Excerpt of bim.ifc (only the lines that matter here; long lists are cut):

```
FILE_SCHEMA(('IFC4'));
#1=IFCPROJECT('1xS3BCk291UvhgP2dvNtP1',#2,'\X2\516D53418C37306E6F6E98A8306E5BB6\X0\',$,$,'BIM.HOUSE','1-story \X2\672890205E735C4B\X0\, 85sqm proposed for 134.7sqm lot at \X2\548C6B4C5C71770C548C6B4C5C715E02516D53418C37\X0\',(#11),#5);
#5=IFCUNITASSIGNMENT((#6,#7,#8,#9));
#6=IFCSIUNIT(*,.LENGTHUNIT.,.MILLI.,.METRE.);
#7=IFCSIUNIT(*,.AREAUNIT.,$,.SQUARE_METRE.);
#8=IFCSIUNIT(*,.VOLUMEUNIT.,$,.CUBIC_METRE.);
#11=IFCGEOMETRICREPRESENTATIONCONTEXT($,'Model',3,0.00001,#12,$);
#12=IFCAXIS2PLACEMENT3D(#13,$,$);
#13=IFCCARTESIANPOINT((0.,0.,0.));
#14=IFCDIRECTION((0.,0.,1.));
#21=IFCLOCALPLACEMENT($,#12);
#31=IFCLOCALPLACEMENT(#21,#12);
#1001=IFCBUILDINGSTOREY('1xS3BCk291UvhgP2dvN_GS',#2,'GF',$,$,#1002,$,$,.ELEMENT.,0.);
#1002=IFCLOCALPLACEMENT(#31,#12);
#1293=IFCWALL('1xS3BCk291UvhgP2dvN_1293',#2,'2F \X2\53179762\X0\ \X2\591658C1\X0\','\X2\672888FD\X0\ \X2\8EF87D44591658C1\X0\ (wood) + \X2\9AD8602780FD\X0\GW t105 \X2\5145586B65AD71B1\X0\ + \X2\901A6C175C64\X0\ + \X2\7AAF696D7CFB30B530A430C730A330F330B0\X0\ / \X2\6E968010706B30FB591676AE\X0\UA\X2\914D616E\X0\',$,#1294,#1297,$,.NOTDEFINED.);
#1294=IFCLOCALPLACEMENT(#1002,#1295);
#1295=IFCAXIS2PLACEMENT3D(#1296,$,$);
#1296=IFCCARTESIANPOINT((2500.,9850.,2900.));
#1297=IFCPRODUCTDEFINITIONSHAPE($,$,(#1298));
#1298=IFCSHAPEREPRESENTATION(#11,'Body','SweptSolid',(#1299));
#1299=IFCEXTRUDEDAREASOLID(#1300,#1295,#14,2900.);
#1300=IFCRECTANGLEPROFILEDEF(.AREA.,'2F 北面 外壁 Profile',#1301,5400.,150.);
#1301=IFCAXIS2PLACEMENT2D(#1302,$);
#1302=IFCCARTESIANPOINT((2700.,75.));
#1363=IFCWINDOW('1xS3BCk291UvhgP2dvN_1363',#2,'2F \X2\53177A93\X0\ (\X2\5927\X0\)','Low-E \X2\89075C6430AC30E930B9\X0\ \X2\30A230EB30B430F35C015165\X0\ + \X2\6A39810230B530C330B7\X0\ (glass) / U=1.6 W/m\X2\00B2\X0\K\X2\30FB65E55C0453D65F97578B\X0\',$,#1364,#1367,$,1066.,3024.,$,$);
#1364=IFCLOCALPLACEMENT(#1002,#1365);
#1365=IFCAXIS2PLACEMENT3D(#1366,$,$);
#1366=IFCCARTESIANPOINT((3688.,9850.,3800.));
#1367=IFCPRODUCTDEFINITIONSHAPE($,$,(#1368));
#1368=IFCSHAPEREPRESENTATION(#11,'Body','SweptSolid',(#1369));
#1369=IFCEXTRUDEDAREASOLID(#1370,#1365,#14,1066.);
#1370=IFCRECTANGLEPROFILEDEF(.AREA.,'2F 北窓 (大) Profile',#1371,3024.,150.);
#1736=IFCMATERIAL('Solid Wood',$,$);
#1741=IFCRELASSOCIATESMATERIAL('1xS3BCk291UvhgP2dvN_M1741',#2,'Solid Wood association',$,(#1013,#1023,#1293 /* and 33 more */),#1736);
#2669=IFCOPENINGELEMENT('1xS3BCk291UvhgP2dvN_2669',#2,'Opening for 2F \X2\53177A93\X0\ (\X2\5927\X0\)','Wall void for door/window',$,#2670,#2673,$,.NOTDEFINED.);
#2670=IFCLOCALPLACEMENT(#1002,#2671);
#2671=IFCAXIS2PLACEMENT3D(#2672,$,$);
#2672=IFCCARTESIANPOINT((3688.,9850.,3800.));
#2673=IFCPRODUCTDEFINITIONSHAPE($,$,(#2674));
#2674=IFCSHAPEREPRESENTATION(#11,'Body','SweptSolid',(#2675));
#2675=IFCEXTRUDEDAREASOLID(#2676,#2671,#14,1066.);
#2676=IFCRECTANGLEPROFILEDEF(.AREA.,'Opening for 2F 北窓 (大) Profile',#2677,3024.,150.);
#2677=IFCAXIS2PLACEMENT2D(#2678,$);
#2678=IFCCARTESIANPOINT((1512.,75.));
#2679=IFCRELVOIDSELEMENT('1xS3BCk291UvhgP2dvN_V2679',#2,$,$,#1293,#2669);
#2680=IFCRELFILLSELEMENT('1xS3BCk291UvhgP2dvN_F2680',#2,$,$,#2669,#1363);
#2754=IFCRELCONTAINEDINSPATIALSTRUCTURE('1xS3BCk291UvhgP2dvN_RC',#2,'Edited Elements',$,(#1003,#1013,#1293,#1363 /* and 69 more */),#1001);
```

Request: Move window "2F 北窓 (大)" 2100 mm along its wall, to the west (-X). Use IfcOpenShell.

```python
import ifcopenshell
import ifcopenshell.api.geometry
import ifcopenshell.util.placement
import ifcopenshell.util.unit

model = ifcopenshell.open("bim.ifc")
unit_scale = ifcopenshell.util.unit.calculate_unit_scale(model)

window = model.by_guid("1xS3BCk291UvhgP2dvN_1363")
opening = window.FillsVoids[0].RelatingOpeningElement
wall = opening.VoidsElements[0].RelatingBuildingElement

wall_matrix = ifcopenshell.util.placement.get_local_placement(wall.ObjectPlacement)
shift = wall_matrix[:3, 0] * -2.1 / unit_scale
before = ifcopenshell.util.placement.get_local_placement(window.ObjectPlacement)[:3, 3].copy()

# The window is not placed relative to its opening, so move both.
for product in (opening, window):
    matrix = ifcopenshell.util.placement.get_local_placement(product.ObjectPlacement)
    matrix[:3, 3] += shift
    ifcopenshell.api.geometry.edit_object_placement(model, product=product, matrix=matrix, is_si=False)

after = ifcopenshell.util.placement.get_local_placement(window.ObjectPlacement)[:3, 3]
print("window moved by", (after - before).round(3) + 0.0)

model.write("bim_updated.ifc")
```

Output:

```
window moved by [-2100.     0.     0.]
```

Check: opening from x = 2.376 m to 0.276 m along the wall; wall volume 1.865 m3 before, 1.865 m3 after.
